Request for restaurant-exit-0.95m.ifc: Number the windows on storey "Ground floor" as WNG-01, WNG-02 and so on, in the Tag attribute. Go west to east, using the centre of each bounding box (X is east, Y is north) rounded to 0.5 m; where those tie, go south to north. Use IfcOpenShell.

First a look at what the model holds.

```python
import ifcopenshell
import ifcopenshell.util.element
import ifcopenshell.util.placement

model = ifcopenshell.open("restaurant-exit-0.95m.ifc")
print(model.schema)
storey = next(s for s in model.by_type("IfcBuildingStorey") if s.Name == "Ground floor")
windows = [e for e in ifcopenshell.util.element.get_decomposition(storey) if e.is_a("IfcWindow")]
for e in sorted(windows, key=lambda e: e.id()):
    origin = ifcopenshell.util.placement.get_local_placement(e.ObjectPlacement)[:3, 3]
    print(e.id(), e.Tag, e.Name, origin.round(2) + 0.0, sep=" | ")
```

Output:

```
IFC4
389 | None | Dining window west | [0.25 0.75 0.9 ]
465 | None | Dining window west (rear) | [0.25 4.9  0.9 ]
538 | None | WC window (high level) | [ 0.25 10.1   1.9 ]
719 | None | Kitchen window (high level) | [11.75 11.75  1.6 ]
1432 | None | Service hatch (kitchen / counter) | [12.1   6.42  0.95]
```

```python
import ifcopenshell
import ifcopenshell.geom
import ifcopenshell.util.element
import ifcopenshell.util.shape

model = ifcopenshell.open("restaurant-exit-0.95m.ifc")
settings = ifcopenshell.geom.settings()
settings.set("use-world-coords", True)


def centre(element):
    shape = ifcopenshell.geom.create_shape(settings, element)
    return ifcopenshell.util.shape.get_bbox_centroid(shape.geometry)


storey = next(s for s in model.by_type("IfcBuildingStorey") if s.Name == "Ground floor")
windows = [e for e in ifcopenshell.util.element.get_decomposition(storey) if e.is_a("IfcWindow")]

# Insertion points can sit at a corner or the storey origin, so sort by the geometry (in metres).
centres = {e: centre(e) for e in windows}
windows.sort(key=lambda e: (round(centres[e][0] / 0.5), centres[e][1]))

for i, e in enumerate(windows, start=1):
    number = f"WNG-{i:02d}"
    e.Tag = number
    print(e.id(), number)

model.write("restaurant-exit-0.95m_v2.ifc")
```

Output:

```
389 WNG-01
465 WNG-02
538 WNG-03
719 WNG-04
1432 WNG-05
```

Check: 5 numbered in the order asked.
